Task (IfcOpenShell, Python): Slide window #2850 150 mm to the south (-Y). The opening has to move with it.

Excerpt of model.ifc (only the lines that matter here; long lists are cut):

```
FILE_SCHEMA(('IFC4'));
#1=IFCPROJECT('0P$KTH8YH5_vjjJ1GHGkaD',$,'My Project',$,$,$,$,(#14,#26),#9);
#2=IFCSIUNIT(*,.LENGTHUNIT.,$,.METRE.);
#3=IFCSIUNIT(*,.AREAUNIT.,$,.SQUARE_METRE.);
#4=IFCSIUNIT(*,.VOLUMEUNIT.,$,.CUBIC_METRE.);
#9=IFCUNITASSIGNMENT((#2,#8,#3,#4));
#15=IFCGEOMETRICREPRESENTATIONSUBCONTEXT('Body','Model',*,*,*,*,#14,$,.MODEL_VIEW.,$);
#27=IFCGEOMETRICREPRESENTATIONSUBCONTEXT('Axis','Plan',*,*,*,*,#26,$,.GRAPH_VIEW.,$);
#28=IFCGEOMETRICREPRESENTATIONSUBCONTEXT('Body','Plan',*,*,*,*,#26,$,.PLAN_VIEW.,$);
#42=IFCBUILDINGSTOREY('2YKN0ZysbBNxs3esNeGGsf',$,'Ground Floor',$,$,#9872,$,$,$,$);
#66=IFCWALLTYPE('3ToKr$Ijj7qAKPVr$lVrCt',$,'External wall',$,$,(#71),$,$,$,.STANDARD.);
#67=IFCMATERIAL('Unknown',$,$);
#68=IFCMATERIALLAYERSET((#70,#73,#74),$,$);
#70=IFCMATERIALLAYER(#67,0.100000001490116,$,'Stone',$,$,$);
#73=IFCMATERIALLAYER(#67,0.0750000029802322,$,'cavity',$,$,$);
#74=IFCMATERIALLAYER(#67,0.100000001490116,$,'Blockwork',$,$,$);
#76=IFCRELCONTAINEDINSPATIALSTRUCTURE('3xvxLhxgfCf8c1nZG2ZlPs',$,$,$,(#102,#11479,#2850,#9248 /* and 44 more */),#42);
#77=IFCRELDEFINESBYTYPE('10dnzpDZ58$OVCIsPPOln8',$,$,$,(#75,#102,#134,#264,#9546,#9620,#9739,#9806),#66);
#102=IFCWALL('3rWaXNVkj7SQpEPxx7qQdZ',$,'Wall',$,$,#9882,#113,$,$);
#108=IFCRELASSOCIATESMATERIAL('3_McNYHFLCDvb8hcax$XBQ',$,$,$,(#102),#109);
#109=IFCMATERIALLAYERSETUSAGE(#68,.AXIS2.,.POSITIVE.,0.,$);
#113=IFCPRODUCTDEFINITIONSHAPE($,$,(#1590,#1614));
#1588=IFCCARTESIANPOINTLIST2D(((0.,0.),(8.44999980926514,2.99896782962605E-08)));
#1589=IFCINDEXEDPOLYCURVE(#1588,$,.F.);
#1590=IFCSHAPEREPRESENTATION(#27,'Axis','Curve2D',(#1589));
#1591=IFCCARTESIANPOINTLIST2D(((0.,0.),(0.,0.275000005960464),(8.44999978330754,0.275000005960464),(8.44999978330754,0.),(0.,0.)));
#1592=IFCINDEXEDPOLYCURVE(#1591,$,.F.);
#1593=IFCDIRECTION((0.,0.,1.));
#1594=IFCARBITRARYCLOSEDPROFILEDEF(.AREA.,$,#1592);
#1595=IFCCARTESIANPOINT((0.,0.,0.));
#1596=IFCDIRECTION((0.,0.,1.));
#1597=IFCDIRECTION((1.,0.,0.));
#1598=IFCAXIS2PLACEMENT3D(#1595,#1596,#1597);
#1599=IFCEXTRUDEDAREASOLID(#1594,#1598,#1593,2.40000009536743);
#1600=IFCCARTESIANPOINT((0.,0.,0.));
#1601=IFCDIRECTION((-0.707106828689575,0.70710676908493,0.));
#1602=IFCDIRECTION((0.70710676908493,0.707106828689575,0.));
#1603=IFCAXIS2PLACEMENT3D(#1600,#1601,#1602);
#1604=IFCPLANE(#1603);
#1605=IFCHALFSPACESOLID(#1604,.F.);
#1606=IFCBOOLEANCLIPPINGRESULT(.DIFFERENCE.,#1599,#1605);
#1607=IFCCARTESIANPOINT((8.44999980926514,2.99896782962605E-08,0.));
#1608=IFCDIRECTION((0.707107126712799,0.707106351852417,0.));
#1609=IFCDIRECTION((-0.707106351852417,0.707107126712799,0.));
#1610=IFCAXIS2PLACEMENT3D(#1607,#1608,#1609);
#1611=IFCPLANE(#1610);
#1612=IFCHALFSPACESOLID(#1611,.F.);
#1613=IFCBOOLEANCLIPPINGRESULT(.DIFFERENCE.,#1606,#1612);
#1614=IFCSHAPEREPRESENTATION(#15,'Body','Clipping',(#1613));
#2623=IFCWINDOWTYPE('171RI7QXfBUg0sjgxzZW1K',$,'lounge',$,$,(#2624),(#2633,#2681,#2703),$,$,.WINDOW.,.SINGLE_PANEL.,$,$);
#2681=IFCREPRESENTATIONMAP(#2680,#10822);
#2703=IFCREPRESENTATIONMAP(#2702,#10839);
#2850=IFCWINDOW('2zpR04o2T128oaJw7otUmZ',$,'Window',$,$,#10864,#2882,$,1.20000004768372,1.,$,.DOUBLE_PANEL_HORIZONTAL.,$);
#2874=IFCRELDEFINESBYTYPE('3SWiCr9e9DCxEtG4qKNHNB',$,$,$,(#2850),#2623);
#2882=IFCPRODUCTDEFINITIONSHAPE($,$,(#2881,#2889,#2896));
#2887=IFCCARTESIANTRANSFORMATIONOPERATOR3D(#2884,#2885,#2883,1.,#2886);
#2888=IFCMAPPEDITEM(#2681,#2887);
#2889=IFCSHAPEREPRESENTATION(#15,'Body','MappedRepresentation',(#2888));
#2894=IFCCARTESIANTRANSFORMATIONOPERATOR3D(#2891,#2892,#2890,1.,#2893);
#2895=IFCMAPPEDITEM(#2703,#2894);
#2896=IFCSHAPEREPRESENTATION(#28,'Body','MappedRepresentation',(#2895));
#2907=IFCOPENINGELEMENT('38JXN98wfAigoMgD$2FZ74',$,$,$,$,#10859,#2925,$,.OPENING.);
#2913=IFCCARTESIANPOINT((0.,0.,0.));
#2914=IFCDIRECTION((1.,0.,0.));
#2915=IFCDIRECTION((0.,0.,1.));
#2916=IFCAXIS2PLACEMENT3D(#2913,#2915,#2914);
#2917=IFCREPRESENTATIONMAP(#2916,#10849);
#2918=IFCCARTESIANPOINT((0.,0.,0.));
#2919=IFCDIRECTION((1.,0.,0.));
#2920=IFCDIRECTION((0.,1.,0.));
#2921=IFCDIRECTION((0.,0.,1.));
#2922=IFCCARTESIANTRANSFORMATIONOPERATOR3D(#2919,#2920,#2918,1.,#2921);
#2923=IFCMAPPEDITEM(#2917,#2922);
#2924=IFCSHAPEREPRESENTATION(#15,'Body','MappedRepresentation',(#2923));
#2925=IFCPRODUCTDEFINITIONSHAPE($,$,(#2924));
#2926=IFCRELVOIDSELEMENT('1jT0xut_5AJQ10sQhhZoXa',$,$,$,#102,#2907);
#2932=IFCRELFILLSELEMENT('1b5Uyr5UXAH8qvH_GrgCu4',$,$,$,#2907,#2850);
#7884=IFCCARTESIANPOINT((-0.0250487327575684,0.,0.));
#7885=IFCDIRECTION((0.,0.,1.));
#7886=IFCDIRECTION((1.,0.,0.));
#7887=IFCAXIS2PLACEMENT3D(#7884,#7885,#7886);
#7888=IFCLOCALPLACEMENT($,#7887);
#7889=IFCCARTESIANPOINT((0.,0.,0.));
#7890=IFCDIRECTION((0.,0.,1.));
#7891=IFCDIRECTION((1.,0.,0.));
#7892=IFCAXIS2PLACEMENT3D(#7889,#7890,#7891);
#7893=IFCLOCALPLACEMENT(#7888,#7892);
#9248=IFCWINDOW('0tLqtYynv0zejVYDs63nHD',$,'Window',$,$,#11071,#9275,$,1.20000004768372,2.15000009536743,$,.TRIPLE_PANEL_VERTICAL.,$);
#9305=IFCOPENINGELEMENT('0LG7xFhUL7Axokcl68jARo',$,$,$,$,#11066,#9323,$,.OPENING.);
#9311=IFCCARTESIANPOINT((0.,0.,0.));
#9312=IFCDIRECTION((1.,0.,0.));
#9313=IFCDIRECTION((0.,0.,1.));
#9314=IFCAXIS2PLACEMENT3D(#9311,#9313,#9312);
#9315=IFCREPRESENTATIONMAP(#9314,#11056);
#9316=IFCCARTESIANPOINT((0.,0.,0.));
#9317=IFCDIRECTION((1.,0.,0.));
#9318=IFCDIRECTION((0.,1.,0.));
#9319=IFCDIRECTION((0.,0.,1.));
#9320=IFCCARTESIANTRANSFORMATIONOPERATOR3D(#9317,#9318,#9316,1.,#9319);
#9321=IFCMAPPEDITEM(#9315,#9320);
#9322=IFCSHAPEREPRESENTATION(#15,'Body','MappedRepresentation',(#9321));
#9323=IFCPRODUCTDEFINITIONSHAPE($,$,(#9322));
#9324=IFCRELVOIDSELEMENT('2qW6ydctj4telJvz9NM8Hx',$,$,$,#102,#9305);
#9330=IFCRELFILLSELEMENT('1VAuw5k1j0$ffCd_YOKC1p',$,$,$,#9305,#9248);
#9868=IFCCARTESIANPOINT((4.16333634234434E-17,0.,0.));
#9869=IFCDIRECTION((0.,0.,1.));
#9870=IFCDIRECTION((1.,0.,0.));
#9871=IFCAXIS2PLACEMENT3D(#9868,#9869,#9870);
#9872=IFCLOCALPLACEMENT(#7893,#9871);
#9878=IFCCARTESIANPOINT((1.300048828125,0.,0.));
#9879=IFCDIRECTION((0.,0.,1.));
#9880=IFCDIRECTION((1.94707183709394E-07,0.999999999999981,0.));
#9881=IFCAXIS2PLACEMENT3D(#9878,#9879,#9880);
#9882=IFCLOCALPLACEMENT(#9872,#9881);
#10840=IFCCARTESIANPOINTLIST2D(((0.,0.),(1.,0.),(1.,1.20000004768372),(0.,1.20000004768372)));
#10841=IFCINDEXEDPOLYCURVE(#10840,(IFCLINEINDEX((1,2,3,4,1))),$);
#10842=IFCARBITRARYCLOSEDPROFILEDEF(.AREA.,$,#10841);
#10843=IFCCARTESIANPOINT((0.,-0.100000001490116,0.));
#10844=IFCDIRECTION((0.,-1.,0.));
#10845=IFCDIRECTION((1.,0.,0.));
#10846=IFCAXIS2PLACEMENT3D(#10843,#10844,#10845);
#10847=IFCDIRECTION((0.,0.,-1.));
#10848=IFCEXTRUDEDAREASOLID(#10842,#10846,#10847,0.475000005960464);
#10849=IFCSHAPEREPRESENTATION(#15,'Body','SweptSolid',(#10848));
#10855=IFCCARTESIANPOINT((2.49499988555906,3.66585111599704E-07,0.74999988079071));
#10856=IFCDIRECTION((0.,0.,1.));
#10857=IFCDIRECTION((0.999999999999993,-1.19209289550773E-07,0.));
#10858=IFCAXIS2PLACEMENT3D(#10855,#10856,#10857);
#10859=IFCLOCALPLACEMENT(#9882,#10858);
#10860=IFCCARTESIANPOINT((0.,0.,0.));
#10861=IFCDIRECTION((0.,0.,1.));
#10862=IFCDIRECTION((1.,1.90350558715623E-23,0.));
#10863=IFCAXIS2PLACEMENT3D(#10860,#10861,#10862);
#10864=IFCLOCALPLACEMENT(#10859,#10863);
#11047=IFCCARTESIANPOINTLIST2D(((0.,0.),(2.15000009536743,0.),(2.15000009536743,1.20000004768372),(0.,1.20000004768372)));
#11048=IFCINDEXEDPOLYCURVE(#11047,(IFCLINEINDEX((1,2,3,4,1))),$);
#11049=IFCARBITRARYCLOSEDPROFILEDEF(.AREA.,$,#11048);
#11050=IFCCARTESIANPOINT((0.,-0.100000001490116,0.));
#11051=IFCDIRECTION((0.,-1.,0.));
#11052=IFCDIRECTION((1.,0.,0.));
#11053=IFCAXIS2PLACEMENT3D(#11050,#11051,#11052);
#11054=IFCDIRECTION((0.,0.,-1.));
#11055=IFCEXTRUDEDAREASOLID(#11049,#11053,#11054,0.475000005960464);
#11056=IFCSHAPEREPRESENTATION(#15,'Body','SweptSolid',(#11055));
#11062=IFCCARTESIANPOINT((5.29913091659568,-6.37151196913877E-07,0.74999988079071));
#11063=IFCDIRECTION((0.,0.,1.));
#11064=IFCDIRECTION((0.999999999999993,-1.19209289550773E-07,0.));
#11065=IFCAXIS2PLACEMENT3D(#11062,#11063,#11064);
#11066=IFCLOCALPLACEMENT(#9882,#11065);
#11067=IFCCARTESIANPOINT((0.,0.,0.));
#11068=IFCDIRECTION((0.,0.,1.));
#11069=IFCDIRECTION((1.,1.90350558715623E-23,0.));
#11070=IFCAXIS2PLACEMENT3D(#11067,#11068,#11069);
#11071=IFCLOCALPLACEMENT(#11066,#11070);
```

```python
import ifcopenshell
import ifcopenshell.api.geometry
import ifcopenshell.util.placement
import ifcopenshell.util.unit

model = ifcopenshell.open("model.ifc")
unit_scale = ifcopenshell.util.unit.calculate_unit_scale(model)

window = model.by_guid("2zpR04o2T128oaJw7otUmZ")
opening = window.FillsVoids[0].RelatingOpeningElement
wall = opening.VoidsElements[0].RelatingBuildingElement

wall_matrix = ifcopenshell.util.placement.get_local_placement(wall.ObjectPlacement)
shift = wall_matrix[:3, 0] * -0.15 / unit_scale
before = ifcopenshell.util.placement.get_local_placement(window.ObjectPlacement)[:3, 3].copy()

# The window is placed relative to its opening, so it follows when the opening moves.
matrix = ifcopenshell.util.placement.get_local_placement(opening.ObjectPlacement)
matrix[:3, 3] += shift
ifcopenshell.api.geometry.edit_object_placement(
    model, product=opening, matrix=matrix, is_si=False, should_transform_children=True
)

after = ifcopenshell.util.placement.get_local_placement(window.ObjectPlacement)[:3, 3]
print("window moved by", (after - before).round(3) + 0.0)

model.write("model_updated.ifc")
```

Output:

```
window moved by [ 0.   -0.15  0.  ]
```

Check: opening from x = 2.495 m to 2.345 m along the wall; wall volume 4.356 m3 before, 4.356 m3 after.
